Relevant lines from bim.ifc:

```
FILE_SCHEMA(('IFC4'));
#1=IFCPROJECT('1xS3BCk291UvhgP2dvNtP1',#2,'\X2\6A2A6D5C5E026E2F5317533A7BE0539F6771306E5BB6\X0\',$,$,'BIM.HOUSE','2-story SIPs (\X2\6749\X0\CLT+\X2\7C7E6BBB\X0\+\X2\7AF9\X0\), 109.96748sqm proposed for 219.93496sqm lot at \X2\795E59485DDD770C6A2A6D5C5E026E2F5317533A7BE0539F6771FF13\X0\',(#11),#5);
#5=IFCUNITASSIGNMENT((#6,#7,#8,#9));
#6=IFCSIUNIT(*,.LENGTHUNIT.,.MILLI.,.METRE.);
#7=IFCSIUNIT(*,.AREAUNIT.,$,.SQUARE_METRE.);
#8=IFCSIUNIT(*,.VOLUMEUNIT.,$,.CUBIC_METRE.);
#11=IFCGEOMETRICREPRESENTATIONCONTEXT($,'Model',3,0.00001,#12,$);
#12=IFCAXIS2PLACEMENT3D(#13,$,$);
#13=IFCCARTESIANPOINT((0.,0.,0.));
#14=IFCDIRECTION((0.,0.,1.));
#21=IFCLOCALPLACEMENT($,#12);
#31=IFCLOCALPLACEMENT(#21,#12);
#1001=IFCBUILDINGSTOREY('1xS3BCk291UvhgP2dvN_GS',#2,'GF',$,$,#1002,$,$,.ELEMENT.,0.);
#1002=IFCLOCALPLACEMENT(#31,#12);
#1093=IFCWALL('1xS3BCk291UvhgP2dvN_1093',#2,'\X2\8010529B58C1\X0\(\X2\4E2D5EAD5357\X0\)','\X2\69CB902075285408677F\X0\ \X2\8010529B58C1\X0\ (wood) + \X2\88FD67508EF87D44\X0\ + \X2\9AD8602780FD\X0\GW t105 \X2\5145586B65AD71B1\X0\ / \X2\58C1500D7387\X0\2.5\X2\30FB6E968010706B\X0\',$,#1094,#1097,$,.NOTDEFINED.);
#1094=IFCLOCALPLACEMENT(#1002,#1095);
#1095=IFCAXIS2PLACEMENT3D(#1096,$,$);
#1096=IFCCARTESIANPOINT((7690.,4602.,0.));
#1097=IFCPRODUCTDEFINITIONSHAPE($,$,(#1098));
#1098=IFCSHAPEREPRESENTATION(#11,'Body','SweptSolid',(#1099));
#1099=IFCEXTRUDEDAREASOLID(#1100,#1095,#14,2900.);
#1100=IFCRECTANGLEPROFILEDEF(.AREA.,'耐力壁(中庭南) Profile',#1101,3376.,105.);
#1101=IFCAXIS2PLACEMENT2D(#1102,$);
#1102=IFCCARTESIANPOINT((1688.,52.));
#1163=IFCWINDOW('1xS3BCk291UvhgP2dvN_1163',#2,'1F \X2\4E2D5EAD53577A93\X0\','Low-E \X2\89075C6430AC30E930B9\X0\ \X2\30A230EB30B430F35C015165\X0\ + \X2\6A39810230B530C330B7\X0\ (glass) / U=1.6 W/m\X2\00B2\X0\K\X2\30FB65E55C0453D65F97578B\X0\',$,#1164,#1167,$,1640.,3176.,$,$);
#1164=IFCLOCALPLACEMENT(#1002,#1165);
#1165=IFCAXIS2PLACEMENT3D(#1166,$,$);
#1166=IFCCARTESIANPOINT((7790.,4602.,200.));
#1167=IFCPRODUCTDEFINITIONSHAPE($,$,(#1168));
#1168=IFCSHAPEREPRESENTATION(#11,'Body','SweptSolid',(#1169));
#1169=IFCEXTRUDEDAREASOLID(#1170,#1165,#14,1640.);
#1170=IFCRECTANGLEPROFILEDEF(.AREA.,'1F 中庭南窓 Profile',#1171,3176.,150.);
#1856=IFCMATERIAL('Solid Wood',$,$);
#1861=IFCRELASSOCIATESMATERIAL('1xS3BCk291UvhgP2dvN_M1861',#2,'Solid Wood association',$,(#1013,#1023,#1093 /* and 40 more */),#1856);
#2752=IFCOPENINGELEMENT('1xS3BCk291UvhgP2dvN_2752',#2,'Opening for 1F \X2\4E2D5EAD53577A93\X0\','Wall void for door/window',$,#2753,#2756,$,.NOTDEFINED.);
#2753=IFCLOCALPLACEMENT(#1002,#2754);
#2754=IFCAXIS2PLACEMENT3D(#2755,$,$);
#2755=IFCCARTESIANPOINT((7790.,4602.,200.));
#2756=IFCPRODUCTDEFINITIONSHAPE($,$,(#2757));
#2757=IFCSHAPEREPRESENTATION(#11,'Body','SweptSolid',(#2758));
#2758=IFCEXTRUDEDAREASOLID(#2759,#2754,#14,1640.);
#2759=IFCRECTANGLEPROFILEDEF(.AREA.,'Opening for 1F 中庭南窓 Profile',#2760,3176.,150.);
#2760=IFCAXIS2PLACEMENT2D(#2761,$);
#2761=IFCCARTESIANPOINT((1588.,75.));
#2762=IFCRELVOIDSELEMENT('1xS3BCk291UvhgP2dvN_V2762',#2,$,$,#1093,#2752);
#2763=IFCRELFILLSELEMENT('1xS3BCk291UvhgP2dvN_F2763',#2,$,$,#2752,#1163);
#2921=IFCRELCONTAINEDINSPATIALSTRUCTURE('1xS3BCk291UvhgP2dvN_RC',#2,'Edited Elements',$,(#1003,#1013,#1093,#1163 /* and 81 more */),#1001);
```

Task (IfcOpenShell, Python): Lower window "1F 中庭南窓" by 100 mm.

```python
import numpy as np
import ifcopenshell
import ifcopenshell.api.geometry
import ifcopenshell.util.placement
import ifcopenshell.util.unit

model = ifcopenshell.open("bim.ifc")
unit_scale = ifcopenshell.util.unit.calculate_unit_scale(model)

window = model.by_guid("1xS3BCk291UvhgP2dvN_1163")
opening = window.FillsVoids[0].RelatingOpeningElement
dz = -100.0

shift = np.array([0.0, 0.0, dz])
# The window is not placed relative to its opening, so move both.
for product in (opening, window):
    matrix = ifcopenshell.util.placement.get_local_placement(product.ObjectPlacement)
    matrix[:3, 3] += shift
    ifcopenshell.api.geometry.edit_object_placement(model, product=product, matrix=matrix, is_si=False)

print(f"moved by {dz * unit_scale:+.3f} m")

model.write("bim-out.ifc")
```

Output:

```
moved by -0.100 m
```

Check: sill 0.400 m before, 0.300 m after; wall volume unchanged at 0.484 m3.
